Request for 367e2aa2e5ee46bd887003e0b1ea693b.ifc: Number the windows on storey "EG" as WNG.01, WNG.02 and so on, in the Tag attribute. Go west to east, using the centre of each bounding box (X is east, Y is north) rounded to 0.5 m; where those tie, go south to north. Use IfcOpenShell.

First a look at what the model holds.

```python
import ifcopenshell
import ifcopenshell.util.element
import ifcopenshell.util.placement

model = ifcopenshell.open("367e2aa2e5ee46bd887003e0b1ea693b.ifc")
print(model.schema)
storey = next(s for s in model.by_type("IfcBuildingStorey") if s.Name == "EG")
windows = [e for e in ifcopenshell.util.element.get_decomposition(storey) if e.is_a("IfcWindow")]
for e in sorted(windows, key=lambda e: e.id()):
    origin = ifcopenshell.util.placement.get_local_placement(e.ObjectPlacement)[:3, 3]
    print(e.id(), e.Tag, e.Name, origin.round(2) + 0.0, sep=" | ")
```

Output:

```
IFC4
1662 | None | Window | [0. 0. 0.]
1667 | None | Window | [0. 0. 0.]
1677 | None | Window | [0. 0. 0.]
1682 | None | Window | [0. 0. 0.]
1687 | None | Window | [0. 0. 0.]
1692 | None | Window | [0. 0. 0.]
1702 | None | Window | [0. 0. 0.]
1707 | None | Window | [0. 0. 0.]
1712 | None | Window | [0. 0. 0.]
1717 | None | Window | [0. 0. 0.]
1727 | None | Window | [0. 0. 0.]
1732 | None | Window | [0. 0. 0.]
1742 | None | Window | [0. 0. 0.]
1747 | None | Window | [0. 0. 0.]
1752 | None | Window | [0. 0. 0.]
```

```python
import ifcopenshell
import ifcopenshell.geom
import ifcopenshell.util.element
import ifcopenshell.util.shape

model = ifcopenshell.open("367e2aa2e5ee46bd887003e0b1ea693b.ifc")
settings = ifcopenshell.geom.settings()
settings.set("use-world-coords", True)


def centre(element):
    shape = ifcopenshell.geom.create_shape(settings, element)
    return ifcopenshell.util.shape.get_bbox_centroid(shape.geometry)


storey = next(s for s in model.by_type("IfcBuildingStorey") if s.Name == "EG")
windows = [e for e in ifcopenshell.util.element.get_decomposition(storey) if e.is_a("IfcWindow")]

# Insertion points can sit at a corner or the storey origin, so sort by the geometry (in metres).
centres = {e: centre(e) for e in windows}
windows.sort(key=lambda e: (round(centres[e][0] / 0.5), centres[e][1]))

for i, e in enumerate(windows, start=1):
    number = f"WNG.{i:02d}"
    e.Tag = number
    print(e.id(), number)

model.write("367e2aa2e5ee46bd887003e0b1ea693b_edited.ifc")
```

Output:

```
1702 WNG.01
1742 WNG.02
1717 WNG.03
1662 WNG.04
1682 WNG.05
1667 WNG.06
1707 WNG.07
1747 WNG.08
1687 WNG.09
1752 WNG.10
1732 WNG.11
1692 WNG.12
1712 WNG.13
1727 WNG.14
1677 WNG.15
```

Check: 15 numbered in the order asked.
